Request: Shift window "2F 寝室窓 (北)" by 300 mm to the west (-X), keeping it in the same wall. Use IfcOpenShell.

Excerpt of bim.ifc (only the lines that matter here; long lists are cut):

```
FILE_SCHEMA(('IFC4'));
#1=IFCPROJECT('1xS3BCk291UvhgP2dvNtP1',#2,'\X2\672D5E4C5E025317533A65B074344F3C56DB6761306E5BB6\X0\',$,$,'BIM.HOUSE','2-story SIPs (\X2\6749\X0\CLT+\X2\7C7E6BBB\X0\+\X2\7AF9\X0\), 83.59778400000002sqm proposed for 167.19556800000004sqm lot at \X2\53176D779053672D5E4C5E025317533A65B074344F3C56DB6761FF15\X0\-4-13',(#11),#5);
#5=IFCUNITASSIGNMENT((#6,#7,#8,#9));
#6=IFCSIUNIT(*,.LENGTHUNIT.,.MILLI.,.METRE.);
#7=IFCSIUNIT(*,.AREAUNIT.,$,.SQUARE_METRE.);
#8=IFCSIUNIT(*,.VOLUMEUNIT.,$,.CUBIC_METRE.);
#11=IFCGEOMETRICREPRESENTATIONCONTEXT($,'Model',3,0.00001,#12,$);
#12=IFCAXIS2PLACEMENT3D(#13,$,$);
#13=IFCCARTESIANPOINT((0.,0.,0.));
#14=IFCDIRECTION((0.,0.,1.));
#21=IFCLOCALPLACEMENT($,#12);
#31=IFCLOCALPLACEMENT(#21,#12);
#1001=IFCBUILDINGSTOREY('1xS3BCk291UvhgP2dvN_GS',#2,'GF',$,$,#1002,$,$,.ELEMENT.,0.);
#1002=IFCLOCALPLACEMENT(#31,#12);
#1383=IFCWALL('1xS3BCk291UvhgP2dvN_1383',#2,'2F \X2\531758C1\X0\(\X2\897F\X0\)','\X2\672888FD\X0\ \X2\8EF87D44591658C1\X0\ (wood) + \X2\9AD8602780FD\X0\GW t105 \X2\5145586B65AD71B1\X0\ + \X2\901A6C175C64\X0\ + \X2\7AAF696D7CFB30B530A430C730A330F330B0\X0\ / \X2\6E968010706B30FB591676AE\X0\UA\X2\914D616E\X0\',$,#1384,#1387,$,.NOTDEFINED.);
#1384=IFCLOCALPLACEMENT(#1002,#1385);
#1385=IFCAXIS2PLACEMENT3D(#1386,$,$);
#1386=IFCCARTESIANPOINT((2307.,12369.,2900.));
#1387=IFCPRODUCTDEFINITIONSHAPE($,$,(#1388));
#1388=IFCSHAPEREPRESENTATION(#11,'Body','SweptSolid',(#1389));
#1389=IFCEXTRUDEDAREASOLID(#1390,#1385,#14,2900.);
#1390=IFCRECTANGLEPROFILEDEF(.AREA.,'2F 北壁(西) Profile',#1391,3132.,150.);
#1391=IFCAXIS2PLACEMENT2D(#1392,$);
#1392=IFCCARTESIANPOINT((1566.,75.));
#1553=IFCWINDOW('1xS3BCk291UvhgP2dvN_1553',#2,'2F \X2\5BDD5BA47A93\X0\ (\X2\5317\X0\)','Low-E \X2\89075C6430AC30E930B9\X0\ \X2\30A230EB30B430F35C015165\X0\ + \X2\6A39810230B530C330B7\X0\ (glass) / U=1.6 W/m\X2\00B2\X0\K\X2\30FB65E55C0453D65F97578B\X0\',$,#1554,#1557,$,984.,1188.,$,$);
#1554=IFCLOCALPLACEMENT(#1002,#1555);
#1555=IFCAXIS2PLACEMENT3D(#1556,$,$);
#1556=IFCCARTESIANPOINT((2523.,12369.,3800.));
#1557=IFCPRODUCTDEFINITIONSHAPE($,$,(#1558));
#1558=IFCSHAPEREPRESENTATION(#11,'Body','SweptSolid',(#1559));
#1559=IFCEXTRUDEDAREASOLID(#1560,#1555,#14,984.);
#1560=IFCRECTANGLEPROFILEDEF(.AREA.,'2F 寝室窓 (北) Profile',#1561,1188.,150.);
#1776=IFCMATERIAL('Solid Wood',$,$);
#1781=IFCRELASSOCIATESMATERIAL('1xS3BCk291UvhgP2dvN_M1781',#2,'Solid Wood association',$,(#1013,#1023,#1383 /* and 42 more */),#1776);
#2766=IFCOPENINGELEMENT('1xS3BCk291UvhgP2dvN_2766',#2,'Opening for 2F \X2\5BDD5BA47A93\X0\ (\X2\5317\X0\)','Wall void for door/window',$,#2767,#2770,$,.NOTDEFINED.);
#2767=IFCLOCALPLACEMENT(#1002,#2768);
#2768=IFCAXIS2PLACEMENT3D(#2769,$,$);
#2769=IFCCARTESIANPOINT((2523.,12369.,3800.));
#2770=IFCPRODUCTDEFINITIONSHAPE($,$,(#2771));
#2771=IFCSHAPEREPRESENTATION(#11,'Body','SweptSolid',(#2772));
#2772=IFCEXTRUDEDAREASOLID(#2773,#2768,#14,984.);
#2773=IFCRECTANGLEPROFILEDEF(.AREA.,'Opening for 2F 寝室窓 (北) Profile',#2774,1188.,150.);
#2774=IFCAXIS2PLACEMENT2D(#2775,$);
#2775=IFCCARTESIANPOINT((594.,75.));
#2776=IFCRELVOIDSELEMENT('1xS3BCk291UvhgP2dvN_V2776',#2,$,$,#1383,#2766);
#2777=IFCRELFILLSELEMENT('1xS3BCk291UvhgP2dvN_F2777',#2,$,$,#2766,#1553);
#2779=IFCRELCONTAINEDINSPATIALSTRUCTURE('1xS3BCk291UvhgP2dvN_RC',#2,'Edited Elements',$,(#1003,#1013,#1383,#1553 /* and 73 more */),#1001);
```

```python
import ifcopenshell
import ifcopenshell.api.geometry
import ifcopenshell.util.placement

model = ifcopenshell.open("bim.ifc")

window = model.by_guid("1xS3BCk291UvhgP2dvN_1553")
opening = window.FillsVoids[0].RelatingOpeningElement
wall = opening.VoidsElements[0].RelatingBuildingElement

wall_matrix = ifcopenshell.util.placement.get_local_placement(wall.ObjectPlacement)
shift = wall_matrix[:3, 0] * -300.0
before = ifcopenshell.util.placement.get_local_placement(window.ObjectPlacement)[:3, 3].copy()

# The window is not placed relative to its opening, so move both.
for product in (opening, window):
    matrix = ifcopenshell.util.placement.get_local_placement(product.ObjectPlacement)
    matrix[:3, 3] += shift
    ifcopenshell.api.geometry.edit_object_placement(model, product=product, matrix=matrix, is_si=False)

after = ifcopenshell.util.placement.get_local_placement(window.ObjectPlacement)[:3, 3]
print("window moved by", (after - before).round(3) + 0.0)

model.write("bim_edited.ifc")
```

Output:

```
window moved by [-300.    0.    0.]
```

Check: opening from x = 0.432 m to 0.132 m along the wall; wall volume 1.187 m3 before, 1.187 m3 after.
